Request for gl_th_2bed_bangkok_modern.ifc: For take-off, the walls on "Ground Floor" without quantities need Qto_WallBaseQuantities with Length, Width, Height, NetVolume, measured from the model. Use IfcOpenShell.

First a look at what the model holds.

```python
import ifcopenshell
import ifcopenshell.util.element
import ifcopenshell.util.unit

model = ifcopenshell.open("gl_th_2bed_bangkok_modern.ifc")
print(model.schema)
for unit_type in ("LENGTHUNIT", "AREAUNIT", "VOLUMEUNIT"):
    print(unit_type, ifcopenshell.util.unit.calculate_unit_scale(model, unit_type))
storey = next(s for s in model.by_type("IfcBuildingStorey") if s.Name == "Ground Floor")
walls = [e for e in ifcopenshell.util.element.get_decomposition(storey) if e.is_a("IfcWall")]
for e in sorted(walls, key=lambda e: e.id()):
    print(e.id(), e.is_a(), e.Name, list(ifcopenshell.util.element.get_psets(e, qtos_only=True)), sep=" | ")
```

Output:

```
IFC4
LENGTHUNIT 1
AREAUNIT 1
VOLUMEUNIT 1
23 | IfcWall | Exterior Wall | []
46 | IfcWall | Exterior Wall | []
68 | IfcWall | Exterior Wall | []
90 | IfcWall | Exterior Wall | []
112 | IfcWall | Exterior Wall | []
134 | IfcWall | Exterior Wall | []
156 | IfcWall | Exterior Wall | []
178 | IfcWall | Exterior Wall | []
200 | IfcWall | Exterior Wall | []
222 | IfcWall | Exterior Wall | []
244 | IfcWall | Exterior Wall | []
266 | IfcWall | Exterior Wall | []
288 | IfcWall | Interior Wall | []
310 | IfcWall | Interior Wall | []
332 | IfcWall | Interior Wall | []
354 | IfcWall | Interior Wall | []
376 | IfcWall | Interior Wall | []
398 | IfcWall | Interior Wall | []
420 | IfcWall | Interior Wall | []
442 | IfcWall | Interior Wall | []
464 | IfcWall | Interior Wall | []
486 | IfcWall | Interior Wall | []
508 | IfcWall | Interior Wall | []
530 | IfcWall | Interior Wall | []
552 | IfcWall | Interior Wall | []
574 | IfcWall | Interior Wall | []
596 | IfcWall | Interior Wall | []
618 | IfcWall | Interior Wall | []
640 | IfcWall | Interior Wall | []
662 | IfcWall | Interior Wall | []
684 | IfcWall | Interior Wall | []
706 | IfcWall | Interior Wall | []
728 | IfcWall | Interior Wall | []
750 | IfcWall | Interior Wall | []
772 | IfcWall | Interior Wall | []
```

```python
import ifcopenshell
import ifcopenshell.api.pset
import ifcopenshell.geom
import ifcopenshell.util.element
import ifcopenshell.util.shape
import ifcopenshell.util.unit

model = ifcopenshell.open("gl_th_2bed_bangkok_modern.ifc")
unit_scale = ifcopenshell.util.unit.calculate_unit_scale(model)
volume_scale = ifcopenshell.util.unit.calculate_unit_scale(model, "VOLUMEUNIT")
settings = ifcopenshell.geom.settings()

storey = next(s for s in model.by_type("IfcBuildingStorey") if s.Name == "Ground Floor")
walls = [e for e in ifcopenshell.util.element.get_decomposition(storey) if e.is_a("IfcWall")]

for e in sorted(walls, key=lambda e: e.id()):
    if ifcopenshell.util.element.get_psets(e, qtos_only=True, should_inherit=False):
        continue
    # Geometry comes back in metres, in the element's own axes.
    shape = ifcopenshell.geom.create_shape(settings, e)
    values = {
        "Length": ifcopenshell.util.shape.get_x(shape.geometry) / unit_scale,
        "Width": ifcopenshell.util.shape.get_y(shape.geometry) / unit_scale,
        "Height": ifcopenshell.util.shape.get_z(shape.geometry) / unit_scale,
        "NetVolume": ifcopenshell.util.shape.get_volume(shape.geometry) / volume_scale,
    }
    qto = ifcopenshell.api.pset.add_qto(model, product=e, name="Qto_WallBaseQuantities")
    ifcopenshell.api.pset.edit_qto(model, qto=qto, properties=values)
    print(e.id(), {k: round(v, 3) for k, v in values.items()})

model.write("gl_th_2bed_bangkok_modern_rev.ifc")
```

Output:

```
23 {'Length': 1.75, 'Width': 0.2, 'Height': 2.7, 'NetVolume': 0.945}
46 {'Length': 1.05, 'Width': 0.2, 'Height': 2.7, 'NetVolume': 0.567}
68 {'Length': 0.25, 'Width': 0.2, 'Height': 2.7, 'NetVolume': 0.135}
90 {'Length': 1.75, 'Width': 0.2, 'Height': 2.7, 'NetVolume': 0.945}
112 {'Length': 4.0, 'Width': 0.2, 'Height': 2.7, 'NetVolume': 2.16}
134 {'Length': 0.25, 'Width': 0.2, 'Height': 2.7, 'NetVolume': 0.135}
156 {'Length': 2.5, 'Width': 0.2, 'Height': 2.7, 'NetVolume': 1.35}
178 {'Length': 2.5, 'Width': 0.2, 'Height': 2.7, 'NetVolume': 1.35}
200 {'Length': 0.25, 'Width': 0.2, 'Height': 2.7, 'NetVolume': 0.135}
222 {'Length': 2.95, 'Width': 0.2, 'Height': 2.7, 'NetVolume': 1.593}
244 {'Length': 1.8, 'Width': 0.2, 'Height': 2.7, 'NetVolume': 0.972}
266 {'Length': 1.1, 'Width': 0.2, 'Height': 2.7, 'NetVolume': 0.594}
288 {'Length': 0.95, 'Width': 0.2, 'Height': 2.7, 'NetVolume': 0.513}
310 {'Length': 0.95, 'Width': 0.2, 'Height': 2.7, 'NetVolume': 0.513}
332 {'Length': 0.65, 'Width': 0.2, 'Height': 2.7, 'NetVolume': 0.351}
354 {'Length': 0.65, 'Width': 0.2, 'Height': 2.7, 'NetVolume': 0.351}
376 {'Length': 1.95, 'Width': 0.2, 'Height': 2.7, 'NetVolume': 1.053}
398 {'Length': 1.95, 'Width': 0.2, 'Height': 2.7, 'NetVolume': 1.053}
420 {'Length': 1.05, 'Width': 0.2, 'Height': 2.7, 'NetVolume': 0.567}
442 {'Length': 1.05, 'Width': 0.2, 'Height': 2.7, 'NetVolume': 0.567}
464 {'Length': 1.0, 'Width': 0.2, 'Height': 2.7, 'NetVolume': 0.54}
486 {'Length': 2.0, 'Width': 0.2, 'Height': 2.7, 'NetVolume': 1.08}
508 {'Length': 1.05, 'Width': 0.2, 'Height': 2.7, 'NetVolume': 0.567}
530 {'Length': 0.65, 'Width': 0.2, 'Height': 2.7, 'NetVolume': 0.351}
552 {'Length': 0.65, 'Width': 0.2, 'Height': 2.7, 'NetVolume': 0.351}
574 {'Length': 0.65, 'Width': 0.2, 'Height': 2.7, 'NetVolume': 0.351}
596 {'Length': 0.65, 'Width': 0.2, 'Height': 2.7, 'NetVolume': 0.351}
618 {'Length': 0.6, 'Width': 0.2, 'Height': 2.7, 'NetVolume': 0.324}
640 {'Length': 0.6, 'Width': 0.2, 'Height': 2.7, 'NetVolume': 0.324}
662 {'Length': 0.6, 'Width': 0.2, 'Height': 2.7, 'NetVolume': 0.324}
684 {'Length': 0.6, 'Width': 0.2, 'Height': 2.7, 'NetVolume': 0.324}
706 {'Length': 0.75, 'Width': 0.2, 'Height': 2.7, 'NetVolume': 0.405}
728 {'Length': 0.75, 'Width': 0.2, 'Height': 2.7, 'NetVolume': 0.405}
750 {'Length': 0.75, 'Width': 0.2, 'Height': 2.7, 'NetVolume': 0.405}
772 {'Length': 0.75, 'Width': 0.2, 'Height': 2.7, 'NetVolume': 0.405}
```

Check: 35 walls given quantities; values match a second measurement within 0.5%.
